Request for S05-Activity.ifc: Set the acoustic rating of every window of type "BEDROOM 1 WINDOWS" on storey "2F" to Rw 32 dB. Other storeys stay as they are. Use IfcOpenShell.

First a look at what the model holds.

```python
import ifcopenshell
import ifcopenshell.util.element

model = ifcopenshell.open("S05-Activity.ifc")
print(model.schema)
storey = next(s for s in model.by_type("IfcBuildingStorey") if s.Name == "2F")
windows = [e for e in ifcopenshell.util.element.get_decomposition(storey) if e.is_a("IfcWindow")]
seen = {}
for e in windows:
    element_type = ifcopenshell.util.element.get_type(e)
    key = (element_type.Name if element_type != e and element_type else None, ifcopenshell.util.element.get_pset(e, "Pset_WindowCommon", "AcousticRating"))
    seen[key] = seen.get(key, 0) + 1
for (name, value), count in sorted(seen.items(), key=str):
    print(count, "x", name, "|", value)
```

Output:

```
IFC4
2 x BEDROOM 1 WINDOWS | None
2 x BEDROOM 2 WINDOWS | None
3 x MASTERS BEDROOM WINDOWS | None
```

```python
import ifcopenshell
import ifcopenshell.api.pset
import ifcopenshell.util.element

model = ifcopenshell.open("S05-Activity.ifc")

storey = next(s for s in model.by_type("IfcBuildingStorey") if s.Name == "2F")
windows = [e for e in ifcopenshell.util.element.get_decomposition(storey) if e.is_a("IfcWindow")]

count = 0
for e in windows:
    element_type = ifcopenshell.util.element.get_type(e)
    if element_type in (None, e) or element_type.Name != "BEDROOM 1 WINDOWS":
        continue
    # add_pset returns the element's existing set when there is one.
    pset = ifcopenshell.api.pset.add_pset(model, product=e, name="Pset_WindowCommon")
    ifcopenshell.api.pset.edit_pset(model, pset=pset, properties={"AcousticRating": "Rw 32 dB"})
    count += 1

print(count, "windows updated")

model.write("S05-Activity_edited.ifc")
```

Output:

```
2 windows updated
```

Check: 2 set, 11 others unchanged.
